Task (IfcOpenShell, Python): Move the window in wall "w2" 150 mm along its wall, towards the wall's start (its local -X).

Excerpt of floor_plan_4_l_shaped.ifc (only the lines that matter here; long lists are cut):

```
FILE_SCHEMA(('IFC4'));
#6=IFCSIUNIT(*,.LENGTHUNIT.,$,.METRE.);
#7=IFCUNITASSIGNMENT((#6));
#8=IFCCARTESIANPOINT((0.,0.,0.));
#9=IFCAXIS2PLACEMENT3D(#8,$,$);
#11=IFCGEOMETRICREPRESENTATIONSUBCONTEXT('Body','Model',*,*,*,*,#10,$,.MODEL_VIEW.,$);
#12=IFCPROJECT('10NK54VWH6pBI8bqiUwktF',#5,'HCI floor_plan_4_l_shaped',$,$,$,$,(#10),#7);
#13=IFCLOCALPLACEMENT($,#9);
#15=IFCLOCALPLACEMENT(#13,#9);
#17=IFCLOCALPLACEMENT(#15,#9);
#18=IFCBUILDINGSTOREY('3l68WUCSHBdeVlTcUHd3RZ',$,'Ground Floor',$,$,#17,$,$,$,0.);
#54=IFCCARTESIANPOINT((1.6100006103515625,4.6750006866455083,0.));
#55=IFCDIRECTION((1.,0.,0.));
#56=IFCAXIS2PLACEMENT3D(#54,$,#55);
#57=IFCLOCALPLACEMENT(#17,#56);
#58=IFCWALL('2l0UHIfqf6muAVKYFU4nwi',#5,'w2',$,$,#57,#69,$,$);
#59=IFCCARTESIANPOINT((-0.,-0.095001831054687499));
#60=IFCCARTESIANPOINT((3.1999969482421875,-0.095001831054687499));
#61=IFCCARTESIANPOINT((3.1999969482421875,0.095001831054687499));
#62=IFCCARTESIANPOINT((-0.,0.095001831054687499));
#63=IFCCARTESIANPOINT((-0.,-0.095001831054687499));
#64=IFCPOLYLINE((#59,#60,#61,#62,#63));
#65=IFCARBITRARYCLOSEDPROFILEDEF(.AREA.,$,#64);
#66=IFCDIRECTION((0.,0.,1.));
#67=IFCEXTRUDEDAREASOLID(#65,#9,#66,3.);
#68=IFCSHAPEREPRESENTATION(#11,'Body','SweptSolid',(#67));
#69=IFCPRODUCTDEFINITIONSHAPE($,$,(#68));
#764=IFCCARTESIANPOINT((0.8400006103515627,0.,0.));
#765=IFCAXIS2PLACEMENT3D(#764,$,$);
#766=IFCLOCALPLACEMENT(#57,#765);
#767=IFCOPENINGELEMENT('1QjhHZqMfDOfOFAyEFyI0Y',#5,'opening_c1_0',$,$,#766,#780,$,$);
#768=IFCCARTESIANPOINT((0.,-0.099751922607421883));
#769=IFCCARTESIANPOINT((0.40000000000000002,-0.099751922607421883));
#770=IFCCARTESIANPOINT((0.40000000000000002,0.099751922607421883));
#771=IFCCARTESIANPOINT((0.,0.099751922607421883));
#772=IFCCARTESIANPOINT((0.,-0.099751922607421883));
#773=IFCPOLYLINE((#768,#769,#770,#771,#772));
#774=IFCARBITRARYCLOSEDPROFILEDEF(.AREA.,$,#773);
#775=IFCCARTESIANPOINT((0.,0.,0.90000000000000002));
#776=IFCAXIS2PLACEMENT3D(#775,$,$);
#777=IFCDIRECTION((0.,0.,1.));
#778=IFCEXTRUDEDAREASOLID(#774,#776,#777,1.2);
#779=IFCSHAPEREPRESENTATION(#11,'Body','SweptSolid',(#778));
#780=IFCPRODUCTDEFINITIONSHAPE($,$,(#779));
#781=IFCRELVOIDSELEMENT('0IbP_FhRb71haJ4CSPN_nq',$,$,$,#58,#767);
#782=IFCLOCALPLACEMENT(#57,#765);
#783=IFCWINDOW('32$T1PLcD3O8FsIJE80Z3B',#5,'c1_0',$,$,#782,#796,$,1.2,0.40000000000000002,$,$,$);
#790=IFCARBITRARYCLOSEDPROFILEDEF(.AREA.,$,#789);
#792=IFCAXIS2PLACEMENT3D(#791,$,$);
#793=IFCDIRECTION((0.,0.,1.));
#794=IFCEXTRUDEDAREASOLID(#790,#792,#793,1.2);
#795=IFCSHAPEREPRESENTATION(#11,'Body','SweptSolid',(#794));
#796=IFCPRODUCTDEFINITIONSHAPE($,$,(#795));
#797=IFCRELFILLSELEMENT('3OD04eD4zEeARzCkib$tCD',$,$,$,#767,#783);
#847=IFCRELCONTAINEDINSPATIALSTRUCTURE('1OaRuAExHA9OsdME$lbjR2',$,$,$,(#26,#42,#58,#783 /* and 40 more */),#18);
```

```python
import ifcopenshell
import ifcopenshell.api.geometry
import ifcopenshell.util.placement

model = ifcopenshell.open("floor_plan_4_l_shaped.ifc")

window = model.by_guid("32$T1PLcD3O8FsIJE80Z3B")
opening = window.FillsVoids[0].RelatingOpeningElement
wall = opening.VoidsElements[0].RelatingBuildingElement

wall_matrix = ifcopenshell.util.placement.get_local_placement(wall.ObjectPlacement)
shift = wall_matrix[:3, 0] * -0.15
before = ifcopenshell.util.placement.get_local_placement(window.ObjectPlacement)[:3, 3].copy()

# The window is not placed relative to its opening, so move both.
for product in (opening, window):
    matrix = ifcopenshell.util.placement.get_local_placement(product.ObjectPlacement)
    matrix[:3, 3] += shift
    ifcopenshell.api.geometry.edit_object_placement(model, product=product, matrix=matrix, is_si=False)

after = ifcopenshell.util.placement.get_local_placement(window.ObjectPlacement)[:3, 3]
print("window moved by", (after - before).round(3) + 0.0)

model.write("floor_plan_4_l_shaped_edited.ifc")
```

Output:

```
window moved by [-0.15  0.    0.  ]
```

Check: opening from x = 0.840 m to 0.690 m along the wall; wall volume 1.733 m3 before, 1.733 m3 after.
